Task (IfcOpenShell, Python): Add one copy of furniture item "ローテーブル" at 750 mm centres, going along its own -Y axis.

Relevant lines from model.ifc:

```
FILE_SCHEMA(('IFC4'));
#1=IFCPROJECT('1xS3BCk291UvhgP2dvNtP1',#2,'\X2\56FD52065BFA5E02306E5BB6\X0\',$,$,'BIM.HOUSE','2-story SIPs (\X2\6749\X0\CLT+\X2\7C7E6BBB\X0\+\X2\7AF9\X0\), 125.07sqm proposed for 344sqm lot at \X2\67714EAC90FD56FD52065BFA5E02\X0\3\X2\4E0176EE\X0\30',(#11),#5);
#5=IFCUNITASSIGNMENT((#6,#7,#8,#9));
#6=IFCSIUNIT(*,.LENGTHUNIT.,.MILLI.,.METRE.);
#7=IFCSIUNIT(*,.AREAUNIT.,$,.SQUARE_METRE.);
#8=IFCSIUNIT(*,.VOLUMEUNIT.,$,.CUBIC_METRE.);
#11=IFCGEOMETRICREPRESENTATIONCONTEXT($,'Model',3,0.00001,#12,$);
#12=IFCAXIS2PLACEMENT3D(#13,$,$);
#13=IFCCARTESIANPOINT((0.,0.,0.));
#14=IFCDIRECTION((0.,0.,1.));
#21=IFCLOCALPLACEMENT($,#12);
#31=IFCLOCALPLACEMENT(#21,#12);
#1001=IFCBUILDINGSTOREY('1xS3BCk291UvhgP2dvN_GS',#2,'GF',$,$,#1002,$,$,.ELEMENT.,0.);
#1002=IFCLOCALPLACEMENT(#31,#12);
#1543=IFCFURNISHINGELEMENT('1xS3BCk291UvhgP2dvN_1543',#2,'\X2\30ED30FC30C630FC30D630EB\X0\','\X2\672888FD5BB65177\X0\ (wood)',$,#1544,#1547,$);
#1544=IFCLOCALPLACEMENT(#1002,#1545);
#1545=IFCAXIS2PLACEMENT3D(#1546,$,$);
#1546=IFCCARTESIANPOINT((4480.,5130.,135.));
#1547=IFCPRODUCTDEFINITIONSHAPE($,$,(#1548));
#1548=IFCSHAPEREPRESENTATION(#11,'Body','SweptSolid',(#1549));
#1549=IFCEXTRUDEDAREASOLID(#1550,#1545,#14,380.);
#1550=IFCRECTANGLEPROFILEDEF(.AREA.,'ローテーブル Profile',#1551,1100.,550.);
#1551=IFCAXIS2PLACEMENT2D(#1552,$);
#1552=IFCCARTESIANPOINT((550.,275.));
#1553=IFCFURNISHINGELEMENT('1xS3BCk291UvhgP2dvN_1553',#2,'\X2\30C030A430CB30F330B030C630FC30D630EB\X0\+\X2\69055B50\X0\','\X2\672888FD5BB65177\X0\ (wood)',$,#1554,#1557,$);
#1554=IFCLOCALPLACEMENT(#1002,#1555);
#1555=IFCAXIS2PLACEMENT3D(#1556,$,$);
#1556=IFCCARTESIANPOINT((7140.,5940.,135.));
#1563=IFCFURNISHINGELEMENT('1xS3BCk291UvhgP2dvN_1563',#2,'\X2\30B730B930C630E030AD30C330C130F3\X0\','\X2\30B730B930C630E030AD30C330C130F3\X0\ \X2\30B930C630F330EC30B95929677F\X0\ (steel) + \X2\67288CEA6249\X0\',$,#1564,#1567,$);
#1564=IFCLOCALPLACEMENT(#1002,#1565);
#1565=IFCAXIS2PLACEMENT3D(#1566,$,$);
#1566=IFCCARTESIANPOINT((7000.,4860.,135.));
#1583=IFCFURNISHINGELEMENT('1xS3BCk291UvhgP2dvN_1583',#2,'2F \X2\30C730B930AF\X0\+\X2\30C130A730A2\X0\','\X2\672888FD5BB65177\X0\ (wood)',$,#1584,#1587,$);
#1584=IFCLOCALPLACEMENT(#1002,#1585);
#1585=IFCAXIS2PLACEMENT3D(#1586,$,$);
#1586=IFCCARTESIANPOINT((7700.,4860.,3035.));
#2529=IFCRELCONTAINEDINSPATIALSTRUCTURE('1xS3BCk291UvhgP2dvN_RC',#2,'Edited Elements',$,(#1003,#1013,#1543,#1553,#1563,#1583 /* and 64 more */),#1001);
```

```python
import ifcopenshell
import ifcopenshell.api.geometry
import ifcopenshell.api.root
import ifcopenshell.util.element
import ifcopenshell.util.placement

model = ifcopenshell.open("model.ifc")


def reuse_history(source, copy):
    """copy_class also copies each property set's owner history, people and application; keep the originals."""
    for rel in copy.IsDefinedBy:
        if rel.is_a("IfcRelDefinesByProperties") and (history := rel.RelatingPropertyDefinition.OwnerHistory):
            rel.RelatingPropertyDefinition.OwnerHistory = source.OwnerHistory
            ifcopenshell.util.element.remove_deep2(model, history)


source = model.by_guid("1xS3BCk291UvhgP2dvN_1543")
base = ifcopenshell.util.placement.get_local_placement(source.ObjectPlacement)
step = -base[:3, 1] * 750.0

for i in range(1, 2):
    copy = ifcopenshell.api.root.copy_class(model, product=source)
    copy.Representation = ifcopenshell.util.element.copy_deep(
        model, source.Representation, exclude=["IfcGeometricRepresentationContext", "IfcRepresentationMap"]
    )
    reuse_history(source, copy)
    matrix = base.copy()
    matrix[:3, 3] += i * step
    print("added at", matrix[:3, 3].round(3) + 0.0)
    ifcopenshell.api.geometry.edit_object_placement(model, product=copy, matrix=matrix, is_si=False)

model.write("model_updated.ifc")
```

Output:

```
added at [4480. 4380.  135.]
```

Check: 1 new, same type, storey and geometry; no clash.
